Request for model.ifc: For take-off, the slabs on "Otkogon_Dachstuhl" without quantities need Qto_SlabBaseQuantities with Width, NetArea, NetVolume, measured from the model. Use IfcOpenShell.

First a look at what the model holds.

```python
import ifcopenshell
import ifcopenshell.util.element
import ifcopenshell.util.unit

model = ifcopenshell.open("model.ifc")
print(model.schema)
for unit_type in ("LENGTHUNIT", "AREAUNIT", "VOLUMEUNIT"):
    print(unit_type, ifcopenshell.util.unit.calculate_unit_scale(model, unit_type))
storey = next(s for s in model.by_type("IfcBuildingStorey") if s.Name == "Otkogon_Dachstuhl")
slabs = [e for e in ifcopenshell.util.element.get_decomposition(storey) if e.is_a("IfcSlab")]
for e in sorted(slabs, key=lambda e: e.id()):
    print(e.id(), e.is_a(), e.Name, list(ifcopenshell.util.element.get_psets(e, qtos_only=True)), sep=" | ")
```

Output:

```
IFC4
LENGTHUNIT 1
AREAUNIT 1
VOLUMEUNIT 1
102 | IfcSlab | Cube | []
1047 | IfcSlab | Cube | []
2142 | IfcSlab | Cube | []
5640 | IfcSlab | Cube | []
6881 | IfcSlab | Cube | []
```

```python
import ifcopenshell
import ifcopenshell.api.pset
import ifcopenshell.geom
import ifcopenshell.util.element
import ifcopenshell.util.shape
import ifcopenshell.util.unit

model = ifcopenshell.open("model.ifc")
unit_scale = ifcopenshell.util.unit.calculate_unit_scale(model)
area_scale = ifcopenshell.util.unit.calculate_unit_scale(model, "AREAUNIT")
volume_scale = ifcopenshell.util.unit.calculate_unit_scale(model, "VOLUMEUNIT")
settings = ifcopenshell.geom.settings()

storey = next(s for s in model.by_type("IfcBuildingStorey") if s.Name == "Otkogon_Dachstuhl")
slabs = [e for e in ifcopenshell.util.element.get_decomposition(storey) if e.is_a("IfcSlab")]

for e in sorted(slabs, key=lambda e: e.id()):
    if ifcopenshell.util.element.get_psets(e, qtos_only=True, should_inherit=False):
        continue
    # Geometry comes back in metres, in the element's own axes.
    shape = ifcopenshell.geom.create_shape(settings, e)
    values = {
        "Width": ifcopenshell.util.shape.get_z(shape.geometry) / unit_scale,
        "NetArea": ifcopenshell.util.shape.get_footprint_area(shape.geometry) / area_scale,
        "NetVolume": ifcopenshell.util.shape.get_volume(shape.geometry) / volume_scale,
    }
    qto = ifcopenshell.api.pset.add_qto(model, product=e, name="Qto_SlabBaseQuantities")
    ifcopenshell.api.pset.edit_qto(model, qto=qto, properties=values)
    print(e.id(), {k: round(v, 3) for k, v in values.items()})

model.write("model-out.ifc")
```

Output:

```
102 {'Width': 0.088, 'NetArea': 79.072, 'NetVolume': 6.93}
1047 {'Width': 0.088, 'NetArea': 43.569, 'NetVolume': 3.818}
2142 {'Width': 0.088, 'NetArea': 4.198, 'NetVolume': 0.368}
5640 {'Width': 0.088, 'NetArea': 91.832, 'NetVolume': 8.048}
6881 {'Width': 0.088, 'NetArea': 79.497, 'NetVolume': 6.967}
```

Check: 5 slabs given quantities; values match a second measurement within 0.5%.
